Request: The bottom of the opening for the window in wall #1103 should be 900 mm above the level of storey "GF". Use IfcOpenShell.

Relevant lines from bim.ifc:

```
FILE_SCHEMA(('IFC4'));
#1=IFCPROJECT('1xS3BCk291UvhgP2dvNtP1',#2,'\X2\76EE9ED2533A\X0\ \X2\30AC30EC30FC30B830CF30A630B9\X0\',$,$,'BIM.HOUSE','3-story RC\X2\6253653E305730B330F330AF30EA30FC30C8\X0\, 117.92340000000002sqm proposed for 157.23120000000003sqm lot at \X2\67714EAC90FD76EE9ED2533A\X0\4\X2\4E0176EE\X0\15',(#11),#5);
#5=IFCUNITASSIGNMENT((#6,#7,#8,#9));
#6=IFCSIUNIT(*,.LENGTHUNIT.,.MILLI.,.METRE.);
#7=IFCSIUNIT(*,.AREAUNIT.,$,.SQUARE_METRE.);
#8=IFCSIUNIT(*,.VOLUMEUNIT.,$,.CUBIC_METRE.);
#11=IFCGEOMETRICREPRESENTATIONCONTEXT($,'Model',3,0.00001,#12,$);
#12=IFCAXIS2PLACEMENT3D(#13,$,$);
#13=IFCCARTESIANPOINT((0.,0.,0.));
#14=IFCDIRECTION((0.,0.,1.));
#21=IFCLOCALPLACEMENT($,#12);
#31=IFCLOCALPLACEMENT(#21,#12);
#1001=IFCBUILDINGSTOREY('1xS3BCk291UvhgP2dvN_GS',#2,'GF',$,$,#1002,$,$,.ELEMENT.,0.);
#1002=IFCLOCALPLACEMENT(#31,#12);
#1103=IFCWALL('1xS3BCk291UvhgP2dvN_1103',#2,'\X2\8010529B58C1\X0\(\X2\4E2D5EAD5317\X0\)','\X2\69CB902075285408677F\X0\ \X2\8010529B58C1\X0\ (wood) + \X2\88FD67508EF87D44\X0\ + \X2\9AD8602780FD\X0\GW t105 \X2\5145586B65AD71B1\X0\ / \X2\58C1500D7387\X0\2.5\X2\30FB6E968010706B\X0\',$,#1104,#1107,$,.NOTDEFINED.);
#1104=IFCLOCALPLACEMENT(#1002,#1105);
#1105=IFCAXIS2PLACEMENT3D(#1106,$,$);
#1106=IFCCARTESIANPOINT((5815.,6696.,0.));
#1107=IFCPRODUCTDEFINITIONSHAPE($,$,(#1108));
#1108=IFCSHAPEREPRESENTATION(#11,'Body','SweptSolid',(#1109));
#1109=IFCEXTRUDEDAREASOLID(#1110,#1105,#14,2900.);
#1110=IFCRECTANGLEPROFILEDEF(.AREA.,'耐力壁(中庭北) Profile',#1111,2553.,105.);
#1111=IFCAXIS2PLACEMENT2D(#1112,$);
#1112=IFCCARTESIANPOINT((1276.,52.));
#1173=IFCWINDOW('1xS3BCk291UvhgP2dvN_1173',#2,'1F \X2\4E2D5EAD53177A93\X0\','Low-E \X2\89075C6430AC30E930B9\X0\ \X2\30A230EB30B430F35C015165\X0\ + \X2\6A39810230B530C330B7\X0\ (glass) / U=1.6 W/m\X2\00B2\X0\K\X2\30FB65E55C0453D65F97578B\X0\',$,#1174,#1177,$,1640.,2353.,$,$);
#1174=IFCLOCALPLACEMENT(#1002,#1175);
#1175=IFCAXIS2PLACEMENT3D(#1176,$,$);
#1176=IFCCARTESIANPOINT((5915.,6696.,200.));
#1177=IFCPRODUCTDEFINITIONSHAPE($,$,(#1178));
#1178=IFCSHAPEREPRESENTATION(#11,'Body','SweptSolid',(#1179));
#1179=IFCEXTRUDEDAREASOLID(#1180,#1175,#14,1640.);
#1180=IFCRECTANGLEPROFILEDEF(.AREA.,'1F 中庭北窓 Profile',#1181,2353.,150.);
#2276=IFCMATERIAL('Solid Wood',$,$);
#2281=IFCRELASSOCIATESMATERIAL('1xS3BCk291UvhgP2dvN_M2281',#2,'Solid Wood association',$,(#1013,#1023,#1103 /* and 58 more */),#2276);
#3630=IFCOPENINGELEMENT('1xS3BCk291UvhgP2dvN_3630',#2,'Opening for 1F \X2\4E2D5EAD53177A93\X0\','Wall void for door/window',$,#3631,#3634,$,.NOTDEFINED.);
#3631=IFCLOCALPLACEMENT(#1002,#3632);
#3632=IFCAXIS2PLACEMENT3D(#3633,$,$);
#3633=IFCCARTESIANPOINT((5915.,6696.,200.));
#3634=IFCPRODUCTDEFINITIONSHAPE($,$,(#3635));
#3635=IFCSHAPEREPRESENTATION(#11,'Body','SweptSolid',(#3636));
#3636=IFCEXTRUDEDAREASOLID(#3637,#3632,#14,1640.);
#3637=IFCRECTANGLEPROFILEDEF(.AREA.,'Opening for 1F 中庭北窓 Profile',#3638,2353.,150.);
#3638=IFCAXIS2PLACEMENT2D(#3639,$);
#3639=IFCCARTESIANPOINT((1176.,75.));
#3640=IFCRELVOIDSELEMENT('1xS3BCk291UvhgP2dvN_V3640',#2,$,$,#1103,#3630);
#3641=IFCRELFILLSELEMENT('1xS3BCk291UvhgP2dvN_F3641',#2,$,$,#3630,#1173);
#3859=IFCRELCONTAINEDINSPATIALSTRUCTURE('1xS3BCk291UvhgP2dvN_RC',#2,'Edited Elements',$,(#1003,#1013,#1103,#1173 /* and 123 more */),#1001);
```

```python
import numpy as np
import ifcopenshell
import ifcopenshell.api.geometry
import ifcopenshell.geom
import ifcopenshell.util.element
import ifcopenshell.util.placement
import ifcopenshell.util.shape
import ifcopenshell.util.unit

model = ifcopenshell.open("bim.ifc")
unit_scale = ifcopenshell.util.unit.calculate_unit_scale(model)

window = model.by_guid("1xS3BCk291UvhgP2dvN_1173")
opening = window.FillsVoids[0].RelatingOpeningElement
storey = ifcopenshell.util.element.get_container(window, ifc_class="IfcBuildingStorey")
level = ifcopenshell.util.placement.get_local_placement(storey.ObjectPlacement)[2, 3]

# The opening's origin need not be at the sill, so measure its lowest point.
shape = ifcopenshell.geom.create_shape(ifcopenshell.geom.settings(), opening)
bottom = ifcopenshell.util.shape.get_shape_bottom_elevation(shape, shape.geometry) / unit_scale
dz = level + 900.0 - bottom

shift = np.array([0.0, 0.0, dz])
# The window is not placed relative to its opening, so move both.
for product in (opening, window):
    matrix = ifcopenshell.util.placement.get_local_placement(product.ObjectPlacement)
    matrix[:3, 3] += shift
    ifcopenshell.api.geometry.edit_object_placement(model, product=product, matrix=matrix, is_si=False)

print(f"moved by {dz * unit_scale:+.3f} m")

model.write("bim-out.ifc")
```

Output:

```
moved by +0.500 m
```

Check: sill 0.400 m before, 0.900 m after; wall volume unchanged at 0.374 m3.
